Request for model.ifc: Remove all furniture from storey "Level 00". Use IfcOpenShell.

First a look at what the model holds.

```python
import ifcopenshell
import ifcopenshell.util.element

model = ifcopenshell.open("model.ifc")
print(model.schema)
storey = next(s for s in model.by_type("IfcBuildingStorey") if s.Name == "Level 00")
furniture = [e for e in ifcopenshell.util.element.get_decomposition(storey) if e.is_a("IfcFurnishingElement")]
seen = {}
for e in furniture:
    element_type = ifcopenshell.util.element.get_type(e)
    name = element_type.Name if element_type not in (None, e) else None
    seen[name] = seen.get(name, 0) + 1
for name, count in sorted(seen.items(), key=str):
    print(count, "x", name)
```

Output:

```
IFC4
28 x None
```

```python
import ifcopenshell
import ifcopenshell.api.root
import ifcopenshell.util.element

model = ifcopenshell.open("model.ifc")

storey = next(s for s in model.by_type("IfcBuildingStorey") if s.Name == "Level 00")
furniture = [e for e in ifcopenshell.util.element.get_decomposition(storey) if e.is_a("IfcFurnishingElement")]

for e in furniture:
    ifcopenshell.api.root.remove_product(model, product=e)
print(len(furniture), "removed")

model.write("model-out.ifc")
```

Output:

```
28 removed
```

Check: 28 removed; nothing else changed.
